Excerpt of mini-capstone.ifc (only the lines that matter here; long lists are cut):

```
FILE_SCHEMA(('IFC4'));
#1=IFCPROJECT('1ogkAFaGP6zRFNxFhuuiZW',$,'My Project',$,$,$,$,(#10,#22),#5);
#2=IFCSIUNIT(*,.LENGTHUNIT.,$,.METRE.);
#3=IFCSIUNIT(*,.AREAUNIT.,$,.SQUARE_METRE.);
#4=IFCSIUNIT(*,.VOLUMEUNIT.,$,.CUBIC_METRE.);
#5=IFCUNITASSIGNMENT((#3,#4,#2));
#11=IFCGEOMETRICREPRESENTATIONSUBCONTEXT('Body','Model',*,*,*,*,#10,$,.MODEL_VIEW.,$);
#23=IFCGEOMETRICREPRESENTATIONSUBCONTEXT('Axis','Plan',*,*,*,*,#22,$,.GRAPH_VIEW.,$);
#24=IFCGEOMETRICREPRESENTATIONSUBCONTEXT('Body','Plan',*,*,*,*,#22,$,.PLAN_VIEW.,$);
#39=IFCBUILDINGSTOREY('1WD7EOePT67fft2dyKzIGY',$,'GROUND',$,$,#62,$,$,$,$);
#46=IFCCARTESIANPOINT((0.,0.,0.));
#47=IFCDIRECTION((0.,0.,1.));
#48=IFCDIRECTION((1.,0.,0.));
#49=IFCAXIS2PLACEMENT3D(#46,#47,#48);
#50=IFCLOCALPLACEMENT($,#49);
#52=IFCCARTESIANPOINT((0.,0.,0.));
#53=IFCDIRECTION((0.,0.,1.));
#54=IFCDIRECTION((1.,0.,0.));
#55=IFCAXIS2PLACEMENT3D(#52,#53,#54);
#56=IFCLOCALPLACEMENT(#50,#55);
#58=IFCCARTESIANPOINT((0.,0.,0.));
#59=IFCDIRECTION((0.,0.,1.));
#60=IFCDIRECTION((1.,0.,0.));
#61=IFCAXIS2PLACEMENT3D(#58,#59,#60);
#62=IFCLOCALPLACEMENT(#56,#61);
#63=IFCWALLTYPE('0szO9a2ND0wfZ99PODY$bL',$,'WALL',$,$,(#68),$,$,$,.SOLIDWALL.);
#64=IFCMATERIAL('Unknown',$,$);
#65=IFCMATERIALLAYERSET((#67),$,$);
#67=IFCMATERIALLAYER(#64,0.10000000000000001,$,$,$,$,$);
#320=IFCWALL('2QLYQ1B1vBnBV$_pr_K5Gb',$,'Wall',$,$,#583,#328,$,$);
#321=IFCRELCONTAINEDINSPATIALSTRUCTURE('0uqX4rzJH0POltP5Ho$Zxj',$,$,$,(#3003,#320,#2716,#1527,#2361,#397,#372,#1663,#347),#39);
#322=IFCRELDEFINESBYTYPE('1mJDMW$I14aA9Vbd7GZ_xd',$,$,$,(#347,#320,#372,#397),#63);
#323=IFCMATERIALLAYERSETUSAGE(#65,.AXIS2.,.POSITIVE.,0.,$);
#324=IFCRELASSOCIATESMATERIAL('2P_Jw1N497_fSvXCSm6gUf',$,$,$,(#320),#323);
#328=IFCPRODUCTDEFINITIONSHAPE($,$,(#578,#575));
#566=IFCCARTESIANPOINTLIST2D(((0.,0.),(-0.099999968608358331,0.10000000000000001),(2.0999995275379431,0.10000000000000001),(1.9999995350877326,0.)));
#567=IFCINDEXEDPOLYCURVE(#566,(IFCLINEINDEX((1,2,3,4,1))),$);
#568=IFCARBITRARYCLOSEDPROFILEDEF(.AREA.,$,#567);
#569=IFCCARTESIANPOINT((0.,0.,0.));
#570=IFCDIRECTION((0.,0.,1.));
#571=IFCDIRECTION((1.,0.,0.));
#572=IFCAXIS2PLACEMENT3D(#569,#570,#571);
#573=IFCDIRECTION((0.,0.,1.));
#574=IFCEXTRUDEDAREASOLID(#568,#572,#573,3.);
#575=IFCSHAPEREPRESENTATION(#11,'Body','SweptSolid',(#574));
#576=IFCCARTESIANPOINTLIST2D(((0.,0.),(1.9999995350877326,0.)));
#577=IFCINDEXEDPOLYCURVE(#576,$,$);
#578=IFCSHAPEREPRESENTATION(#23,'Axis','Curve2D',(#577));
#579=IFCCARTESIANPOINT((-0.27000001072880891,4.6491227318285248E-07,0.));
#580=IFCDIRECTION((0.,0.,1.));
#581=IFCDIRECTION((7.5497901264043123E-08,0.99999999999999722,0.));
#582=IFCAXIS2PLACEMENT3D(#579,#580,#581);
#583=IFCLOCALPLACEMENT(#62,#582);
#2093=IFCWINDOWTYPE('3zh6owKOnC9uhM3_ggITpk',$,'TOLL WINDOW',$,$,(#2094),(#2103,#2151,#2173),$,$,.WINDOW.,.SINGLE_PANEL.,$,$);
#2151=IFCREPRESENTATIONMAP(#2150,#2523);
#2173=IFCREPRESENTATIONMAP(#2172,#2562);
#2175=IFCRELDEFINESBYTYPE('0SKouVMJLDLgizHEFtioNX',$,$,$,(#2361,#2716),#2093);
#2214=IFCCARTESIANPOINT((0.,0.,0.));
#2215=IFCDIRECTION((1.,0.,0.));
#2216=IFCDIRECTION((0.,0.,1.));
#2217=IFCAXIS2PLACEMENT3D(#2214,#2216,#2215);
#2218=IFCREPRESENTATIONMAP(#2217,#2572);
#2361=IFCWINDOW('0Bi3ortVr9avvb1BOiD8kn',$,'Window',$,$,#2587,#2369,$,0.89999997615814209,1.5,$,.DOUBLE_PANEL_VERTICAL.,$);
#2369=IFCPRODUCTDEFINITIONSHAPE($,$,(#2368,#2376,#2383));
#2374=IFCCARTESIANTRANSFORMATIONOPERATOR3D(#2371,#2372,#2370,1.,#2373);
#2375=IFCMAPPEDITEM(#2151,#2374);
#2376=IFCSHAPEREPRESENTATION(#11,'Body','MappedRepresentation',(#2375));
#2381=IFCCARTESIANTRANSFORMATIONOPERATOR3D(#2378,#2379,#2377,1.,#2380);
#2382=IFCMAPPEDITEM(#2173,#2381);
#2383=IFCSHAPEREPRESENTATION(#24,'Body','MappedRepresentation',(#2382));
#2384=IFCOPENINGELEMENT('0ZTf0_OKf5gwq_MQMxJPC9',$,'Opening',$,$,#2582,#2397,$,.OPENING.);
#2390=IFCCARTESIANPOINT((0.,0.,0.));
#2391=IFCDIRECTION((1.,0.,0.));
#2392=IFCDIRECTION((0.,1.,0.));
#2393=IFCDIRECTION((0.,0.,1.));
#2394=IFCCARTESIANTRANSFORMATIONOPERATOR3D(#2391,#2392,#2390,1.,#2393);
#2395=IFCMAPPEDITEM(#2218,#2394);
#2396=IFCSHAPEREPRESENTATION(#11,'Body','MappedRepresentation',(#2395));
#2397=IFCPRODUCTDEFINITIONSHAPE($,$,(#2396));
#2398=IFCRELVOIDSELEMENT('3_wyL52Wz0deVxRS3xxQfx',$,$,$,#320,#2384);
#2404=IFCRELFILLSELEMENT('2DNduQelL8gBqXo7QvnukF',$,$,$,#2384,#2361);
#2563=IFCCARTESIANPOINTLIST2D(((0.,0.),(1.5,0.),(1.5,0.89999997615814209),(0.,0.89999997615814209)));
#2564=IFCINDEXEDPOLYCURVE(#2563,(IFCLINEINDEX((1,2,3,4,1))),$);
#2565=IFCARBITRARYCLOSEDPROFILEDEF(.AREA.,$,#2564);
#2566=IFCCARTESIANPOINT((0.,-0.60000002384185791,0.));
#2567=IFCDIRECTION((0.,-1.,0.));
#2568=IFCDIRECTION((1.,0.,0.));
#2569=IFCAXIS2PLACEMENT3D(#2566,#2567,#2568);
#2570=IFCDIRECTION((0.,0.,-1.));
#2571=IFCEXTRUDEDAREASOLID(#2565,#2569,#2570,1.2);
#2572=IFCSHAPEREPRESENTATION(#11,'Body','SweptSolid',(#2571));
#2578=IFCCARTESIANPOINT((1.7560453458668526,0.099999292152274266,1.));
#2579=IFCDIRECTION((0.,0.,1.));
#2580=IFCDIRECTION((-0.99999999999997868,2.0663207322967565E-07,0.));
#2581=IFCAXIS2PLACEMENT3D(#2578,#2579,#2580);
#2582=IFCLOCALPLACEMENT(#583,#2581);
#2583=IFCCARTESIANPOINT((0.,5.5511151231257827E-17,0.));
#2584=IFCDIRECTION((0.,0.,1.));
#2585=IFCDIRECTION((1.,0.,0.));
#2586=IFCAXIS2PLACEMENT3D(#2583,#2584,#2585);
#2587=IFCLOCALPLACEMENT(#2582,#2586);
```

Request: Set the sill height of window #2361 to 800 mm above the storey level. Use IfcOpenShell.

```python
import numpy as np
import ifcopenshell
import ifcopenshell.api.geometry
import ifcopenshell.geom
import ifcopenshell.util.element
import ifcopenshell.util.placement
import ifcopenshell.util.shape
import ifcopenshell.util.unit

model = ifcopenshell.open("mini-capstone.ifc")
unit_scale = ifcopenshell.util.unit.calculate_unit_scale(model)

window = model.by_guid("0Bi3ortVr9avvb1BOiD8kn")
opening = window.FillsVoids[0].RelatingOpeningElement
storey = ifcopenshell.util.element.get_container(window, ifc_class="IfcBuildingStorey")
level = ifcopenshell.util.placement.get_local_placement(storey.ObjectPlacement)[2, 3]

# The opening's origin need not be at the sill, so measure its lowest point.
shape = ifcopenshell.geom.create_shape(ifcopenshell.geom.settings(), opening)
bottom = ifcopenshell.util.shape.get_shape_bottom_elevation(shape, shape.geometry) / unit_scale
dz = level + 0.8 / unit_scale - bottom

shift = np.array([0.0, 0.0, dz])
# The window is placed relative to its opening, so it follows when the opening moves.
matrix = ifcopenshell.util.placement.get_local_placement(opening.ObjectPlacement)
matrix[:3, 3] += shift
ifcopenshell.api.geometry.edit_object_placement(
    model, product=opening, matrix=matrix, is_si=False, should_transform_children=True
)

print(f"moved by {dz * unit_scale:+.3f} m")

model.write("mini-capstone_edited.ifc")
```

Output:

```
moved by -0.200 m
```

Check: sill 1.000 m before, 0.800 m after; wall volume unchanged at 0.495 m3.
